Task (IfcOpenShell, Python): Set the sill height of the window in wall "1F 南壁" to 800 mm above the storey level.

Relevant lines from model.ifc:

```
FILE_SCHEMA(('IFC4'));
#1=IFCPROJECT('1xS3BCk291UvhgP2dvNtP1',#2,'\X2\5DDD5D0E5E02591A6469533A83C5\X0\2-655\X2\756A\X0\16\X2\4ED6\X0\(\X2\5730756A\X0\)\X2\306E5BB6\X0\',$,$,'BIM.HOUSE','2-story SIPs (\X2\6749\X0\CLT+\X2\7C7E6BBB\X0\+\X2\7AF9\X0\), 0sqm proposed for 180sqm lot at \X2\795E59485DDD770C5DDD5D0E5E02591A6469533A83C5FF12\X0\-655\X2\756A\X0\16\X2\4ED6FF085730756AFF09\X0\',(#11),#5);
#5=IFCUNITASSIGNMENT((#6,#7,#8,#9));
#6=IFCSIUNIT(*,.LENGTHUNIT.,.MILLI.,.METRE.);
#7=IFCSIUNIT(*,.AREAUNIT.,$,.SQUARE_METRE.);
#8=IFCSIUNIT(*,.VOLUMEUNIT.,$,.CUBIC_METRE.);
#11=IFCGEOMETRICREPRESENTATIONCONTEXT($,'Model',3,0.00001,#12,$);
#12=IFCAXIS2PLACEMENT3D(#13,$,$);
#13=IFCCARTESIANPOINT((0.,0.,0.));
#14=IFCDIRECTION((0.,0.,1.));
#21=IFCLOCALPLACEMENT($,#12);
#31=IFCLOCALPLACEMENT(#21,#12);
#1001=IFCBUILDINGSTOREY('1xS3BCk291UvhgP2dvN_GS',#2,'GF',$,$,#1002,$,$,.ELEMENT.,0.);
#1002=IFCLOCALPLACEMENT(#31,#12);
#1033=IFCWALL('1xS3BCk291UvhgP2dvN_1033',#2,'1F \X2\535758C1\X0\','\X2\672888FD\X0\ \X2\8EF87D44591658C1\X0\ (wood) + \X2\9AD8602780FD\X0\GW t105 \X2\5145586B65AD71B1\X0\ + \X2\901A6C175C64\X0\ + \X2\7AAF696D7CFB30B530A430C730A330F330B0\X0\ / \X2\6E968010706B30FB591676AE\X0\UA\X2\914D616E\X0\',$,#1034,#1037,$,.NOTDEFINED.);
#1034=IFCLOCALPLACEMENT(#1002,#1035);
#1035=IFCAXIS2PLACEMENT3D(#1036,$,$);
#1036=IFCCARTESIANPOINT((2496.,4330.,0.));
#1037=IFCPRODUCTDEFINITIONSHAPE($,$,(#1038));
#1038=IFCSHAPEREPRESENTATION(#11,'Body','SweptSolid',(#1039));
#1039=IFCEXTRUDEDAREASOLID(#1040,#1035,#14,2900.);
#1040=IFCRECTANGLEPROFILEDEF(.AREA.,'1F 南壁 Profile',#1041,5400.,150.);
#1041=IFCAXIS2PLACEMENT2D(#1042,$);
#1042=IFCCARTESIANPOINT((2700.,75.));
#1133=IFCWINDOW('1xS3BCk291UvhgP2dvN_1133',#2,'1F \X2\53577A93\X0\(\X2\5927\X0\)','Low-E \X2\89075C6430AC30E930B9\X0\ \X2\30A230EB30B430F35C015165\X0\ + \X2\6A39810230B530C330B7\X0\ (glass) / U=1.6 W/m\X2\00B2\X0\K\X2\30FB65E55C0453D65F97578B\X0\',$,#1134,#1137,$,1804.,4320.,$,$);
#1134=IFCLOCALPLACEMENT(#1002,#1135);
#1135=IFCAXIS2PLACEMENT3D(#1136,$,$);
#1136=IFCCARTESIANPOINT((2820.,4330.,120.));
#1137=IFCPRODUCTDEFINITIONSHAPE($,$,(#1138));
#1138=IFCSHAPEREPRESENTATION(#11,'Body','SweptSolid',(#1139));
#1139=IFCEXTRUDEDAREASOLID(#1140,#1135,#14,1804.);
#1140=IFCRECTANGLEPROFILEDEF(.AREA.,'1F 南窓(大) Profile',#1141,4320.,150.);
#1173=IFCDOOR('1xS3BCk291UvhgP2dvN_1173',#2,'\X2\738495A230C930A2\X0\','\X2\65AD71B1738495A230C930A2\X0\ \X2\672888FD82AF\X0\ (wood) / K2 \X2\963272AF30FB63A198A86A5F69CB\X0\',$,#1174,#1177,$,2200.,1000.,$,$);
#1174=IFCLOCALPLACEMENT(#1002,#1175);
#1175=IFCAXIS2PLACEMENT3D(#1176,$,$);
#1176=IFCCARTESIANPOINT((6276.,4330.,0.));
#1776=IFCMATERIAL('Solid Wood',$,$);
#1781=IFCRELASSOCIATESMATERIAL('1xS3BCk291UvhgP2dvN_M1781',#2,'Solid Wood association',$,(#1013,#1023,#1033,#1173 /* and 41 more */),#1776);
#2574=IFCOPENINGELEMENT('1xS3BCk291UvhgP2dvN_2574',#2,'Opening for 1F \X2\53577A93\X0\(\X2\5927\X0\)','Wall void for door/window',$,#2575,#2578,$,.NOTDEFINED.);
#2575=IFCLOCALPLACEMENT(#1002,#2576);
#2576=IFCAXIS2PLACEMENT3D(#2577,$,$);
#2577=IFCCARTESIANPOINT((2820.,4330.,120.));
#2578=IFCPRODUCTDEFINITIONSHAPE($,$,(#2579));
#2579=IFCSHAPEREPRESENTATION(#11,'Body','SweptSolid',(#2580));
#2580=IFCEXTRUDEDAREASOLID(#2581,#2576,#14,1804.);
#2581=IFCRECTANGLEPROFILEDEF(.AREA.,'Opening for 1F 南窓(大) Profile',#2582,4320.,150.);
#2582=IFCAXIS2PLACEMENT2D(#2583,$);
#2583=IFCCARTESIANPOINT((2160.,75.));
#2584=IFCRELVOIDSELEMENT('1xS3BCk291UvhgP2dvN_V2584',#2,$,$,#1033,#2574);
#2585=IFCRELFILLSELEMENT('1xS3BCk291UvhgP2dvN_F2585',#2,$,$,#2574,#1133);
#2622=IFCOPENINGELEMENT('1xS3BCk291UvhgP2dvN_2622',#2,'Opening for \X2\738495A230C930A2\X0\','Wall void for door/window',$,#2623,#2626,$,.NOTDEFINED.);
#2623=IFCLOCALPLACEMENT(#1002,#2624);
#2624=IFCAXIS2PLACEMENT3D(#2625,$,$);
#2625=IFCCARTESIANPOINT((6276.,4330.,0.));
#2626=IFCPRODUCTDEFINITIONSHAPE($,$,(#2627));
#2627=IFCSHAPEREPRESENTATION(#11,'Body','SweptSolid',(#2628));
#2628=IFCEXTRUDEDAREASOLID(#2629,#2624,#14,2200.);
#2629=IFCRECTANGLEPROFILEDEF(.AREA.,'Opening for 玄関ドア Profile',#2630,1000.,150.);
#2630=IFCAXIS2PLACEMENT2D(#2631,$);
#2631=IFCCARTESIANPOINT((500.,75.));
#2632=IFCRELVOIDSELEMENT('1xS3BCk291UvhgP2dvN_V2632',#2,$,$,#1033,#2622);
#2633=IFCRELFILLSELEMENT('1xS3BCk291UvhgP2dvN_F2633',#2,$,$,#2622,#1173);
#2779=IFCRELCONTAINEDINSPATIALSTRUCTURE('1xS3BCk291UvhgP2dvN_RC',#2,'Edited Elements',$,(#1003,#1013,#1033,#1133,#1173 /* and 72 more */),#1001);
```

```python
import numpy as np
import ifcopenshell
import ifcopenshell.api.geometry
import ifcopenshell.geom
import ifcopenshell.util.element
import ifcopenshell.util.placement
import ifcopenshell.util.shape
import ifcopenshell.util.unit

model = ifcopenshell.open("model.ifc")
unit_scale = ifcopenshell.util.unit.calculate_unit_scale(model)

window = model.by_guid("1xS3BCk291UvhgP2dvN_1133")
opening = window.FillsVoids[0].RelatingOpeningElement
storey = ifcopenshell.util.element.get_container(window, ifc_class="IfcBuildingStorey")
level = ifcopenshell.util.placement.get_local_placement(storey.ObjectPlacement)[2, 3]

# The opening's origin need not be at the sill, so measure its lowest point.
shape = ifcopenshell.geom.create_shape(ifcopenshell.geom.settings(), opening)
bottom = ifcopenshell.util.shape.get_shape_bottom_elevation(shape, shape.geometry) / unit_scale
dz = level + 800.0 - bottom

shift = np.array([0.0, 0.0, dz])
# The window is not placed relative to its opening, so move both.
for product in (opening, window):
    matrix = ifcopenshell.util.placement.get_local_placement(product.ObjectPlacement)
    matrix[:3, 3] += shift
    ifcopenshell.api.geometry.edit_object_placement(model, product=product, matrix=matrix, is_si=False)

print(f"moved by {dz * unit_scale:+.3f} m")

model.write("model_edited.ifc")
```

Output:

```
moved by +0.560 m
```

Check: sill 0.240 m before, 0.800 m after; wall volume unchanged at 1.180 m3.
